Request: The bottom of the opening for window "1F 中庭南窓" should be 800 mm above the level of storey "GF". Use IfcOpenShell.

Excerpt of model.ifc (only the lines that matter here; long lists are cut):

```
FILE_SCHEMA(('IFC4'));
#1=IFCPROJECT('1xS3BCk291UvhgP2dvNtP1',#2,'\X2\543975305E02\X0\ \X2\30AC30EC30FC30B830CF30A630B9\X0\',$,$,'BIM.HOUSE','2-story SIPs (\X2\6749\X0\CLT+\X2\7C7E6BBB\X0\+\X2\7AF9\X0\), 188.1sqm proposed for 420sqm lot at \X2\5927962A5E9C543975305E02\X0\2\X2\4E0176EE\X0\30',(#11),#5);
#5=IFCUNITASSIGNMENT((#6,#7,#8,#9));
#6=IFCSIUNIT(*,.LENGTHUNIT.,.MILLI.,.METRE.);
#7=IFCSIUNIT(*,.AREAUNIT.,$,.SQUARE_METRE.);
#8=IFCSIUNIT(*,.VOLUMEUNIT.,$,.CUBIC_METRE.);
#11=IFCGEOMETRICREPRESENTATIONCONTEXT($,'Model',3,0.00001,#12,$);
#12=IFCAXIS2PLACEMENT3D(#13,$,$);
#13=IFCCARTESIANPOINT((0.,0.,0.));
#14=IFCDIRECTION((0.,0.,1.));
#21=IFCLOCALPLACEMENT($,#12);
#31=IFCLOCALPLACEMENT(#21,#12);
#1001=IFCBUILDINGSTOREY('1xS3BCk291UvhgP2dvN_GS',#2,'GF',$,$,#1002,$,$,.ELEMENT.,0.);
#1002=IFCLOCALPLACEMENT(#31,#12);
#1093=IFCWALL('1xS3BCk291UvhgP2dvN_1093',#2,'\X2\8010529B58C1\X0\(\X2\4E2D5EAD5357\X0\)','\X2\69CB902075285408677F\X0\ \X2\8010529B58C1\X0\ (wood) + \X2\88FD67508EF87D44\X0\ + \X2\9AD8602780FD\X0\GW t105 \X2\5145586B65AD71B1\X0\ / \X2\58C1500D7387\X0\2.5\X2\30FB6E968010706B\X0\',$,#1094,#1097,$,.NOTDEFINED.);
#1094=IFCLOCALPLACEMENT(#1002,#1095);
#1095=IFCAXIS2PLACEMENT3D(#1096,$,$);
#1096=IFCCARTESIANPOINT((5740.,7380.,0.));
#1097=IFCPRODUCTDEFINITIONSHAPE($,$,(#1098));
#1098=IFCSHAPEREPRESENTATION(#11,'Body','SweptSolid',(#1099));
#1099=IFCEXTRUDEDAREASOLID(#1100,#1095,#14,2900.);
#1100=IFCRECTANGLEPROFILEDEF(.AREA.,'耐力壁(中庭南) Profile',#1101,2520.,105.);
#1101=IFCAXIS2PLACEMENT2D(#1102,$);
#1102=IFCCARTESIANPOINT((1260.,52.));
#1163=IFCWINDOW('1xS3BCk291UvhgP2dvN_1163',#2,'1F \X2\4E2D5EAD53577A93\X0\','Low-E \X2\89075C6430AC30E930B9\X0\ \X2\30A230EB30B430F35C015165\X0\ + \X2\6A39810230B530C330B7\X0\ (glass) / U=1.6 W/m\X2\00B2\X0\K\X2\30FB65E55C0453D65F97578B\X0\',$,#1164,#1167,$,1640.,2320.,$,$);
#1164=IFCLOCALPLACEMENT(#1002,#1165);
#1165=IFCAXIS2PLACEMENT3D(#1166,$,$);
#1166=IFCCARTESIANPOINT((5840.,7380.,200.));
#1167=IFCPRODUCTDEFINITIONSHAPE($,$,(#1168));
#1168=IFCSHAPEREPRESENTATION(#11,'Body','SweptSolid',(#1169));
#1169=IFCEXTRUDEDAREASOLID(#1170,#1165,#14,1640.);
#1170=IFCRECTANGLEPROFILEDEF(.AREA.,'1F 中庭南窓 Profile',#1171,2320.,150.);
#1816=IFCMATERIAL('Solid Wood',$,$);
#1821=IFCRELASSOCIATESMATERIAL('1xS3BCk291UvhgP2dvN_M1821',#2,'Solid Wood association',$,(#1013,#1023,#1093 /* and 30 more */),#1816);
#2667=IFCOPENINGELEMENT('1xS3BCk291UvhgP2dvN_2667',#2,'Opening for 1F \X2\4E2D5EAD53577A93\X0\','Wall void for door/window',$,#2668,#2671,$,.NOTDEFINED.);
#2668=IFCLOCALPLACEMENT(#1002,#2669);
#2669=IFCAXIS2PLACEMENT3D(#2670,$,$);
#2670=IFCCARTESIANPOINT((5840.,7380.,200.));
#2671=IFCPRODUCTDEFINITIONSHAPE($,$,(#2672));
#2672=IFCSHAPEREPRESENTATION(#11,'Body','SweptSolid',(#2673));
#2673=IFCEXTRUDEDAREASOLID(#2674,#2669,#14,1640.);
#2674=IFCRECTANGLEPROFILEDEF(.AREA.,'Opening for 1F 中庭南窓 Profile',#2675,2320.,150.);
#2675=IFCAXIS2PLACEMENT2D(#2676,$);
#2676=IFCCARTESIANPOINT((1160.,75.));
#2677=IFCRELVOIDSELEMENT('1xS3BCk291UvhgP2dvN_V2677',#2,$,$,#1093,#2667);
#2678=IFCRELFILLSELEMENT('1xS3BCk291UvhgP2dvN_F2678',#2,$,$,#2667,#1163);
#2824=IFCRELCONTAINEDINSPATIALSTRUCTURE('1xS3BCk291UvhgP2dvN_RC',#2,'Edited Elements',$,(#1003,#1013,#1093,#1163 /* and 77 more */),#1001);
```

```python
import numpy as np
import ifcopenshell
import ifcopenshell.api.geometry
import ifcopenshell.geom
import ifcopenshell.util.element
import ifcopenshell.util.placement
import ifcopenshell.util.shape
import ifcopenshell.util.unit

model = ifcopenshell.open("model.ifc")
unit_scale = ifcopenshell.util.unit.calculate_unit_scale(model)

window = model.by_guid("1xS3BCk291UvhgP2dvN_1163")
opening = window.FillsVoids[0].RelatingOpeningElement
storey = ifcopenshell.util.element.get_container(window, ifc_class="IfcBuildingStorey")
level = ifcopenshell.util.placement.get_local_placement(storey.ObjectPlacement)[2, 3]

# The opening's origin need not be at the sill, so measure its lowest point.
shape = ifcopenshell.geom.create_shape(ifcopenshell.geom.settings(), opening)
bottom = ifcopenshell.util.shape.get_shape_bottom_elevation(shape, shape.geometry) / unit_scale
dz = level + 0.8 / unit_scale - bottom

shift = np.array([0.0, 0.0, dz])
# The window is not placed relative to its opening, so move both.
for product in (opening, window):
    matrix = ifcopenshell.util.placement.get_local_placement(product.ObjectPlacement)
    matrix[:3, 3] += shift
    ifcopenshell.api.geometry.edit_object_placement(model, product=product, matrix=matrix, is_si=False)

print(f"moved by {dz * unit_scale:+.3f} m")

model.write("model_updated.ifc")
```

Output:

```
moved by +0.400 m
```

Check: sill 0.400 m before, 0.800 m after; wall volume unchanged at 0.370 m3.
